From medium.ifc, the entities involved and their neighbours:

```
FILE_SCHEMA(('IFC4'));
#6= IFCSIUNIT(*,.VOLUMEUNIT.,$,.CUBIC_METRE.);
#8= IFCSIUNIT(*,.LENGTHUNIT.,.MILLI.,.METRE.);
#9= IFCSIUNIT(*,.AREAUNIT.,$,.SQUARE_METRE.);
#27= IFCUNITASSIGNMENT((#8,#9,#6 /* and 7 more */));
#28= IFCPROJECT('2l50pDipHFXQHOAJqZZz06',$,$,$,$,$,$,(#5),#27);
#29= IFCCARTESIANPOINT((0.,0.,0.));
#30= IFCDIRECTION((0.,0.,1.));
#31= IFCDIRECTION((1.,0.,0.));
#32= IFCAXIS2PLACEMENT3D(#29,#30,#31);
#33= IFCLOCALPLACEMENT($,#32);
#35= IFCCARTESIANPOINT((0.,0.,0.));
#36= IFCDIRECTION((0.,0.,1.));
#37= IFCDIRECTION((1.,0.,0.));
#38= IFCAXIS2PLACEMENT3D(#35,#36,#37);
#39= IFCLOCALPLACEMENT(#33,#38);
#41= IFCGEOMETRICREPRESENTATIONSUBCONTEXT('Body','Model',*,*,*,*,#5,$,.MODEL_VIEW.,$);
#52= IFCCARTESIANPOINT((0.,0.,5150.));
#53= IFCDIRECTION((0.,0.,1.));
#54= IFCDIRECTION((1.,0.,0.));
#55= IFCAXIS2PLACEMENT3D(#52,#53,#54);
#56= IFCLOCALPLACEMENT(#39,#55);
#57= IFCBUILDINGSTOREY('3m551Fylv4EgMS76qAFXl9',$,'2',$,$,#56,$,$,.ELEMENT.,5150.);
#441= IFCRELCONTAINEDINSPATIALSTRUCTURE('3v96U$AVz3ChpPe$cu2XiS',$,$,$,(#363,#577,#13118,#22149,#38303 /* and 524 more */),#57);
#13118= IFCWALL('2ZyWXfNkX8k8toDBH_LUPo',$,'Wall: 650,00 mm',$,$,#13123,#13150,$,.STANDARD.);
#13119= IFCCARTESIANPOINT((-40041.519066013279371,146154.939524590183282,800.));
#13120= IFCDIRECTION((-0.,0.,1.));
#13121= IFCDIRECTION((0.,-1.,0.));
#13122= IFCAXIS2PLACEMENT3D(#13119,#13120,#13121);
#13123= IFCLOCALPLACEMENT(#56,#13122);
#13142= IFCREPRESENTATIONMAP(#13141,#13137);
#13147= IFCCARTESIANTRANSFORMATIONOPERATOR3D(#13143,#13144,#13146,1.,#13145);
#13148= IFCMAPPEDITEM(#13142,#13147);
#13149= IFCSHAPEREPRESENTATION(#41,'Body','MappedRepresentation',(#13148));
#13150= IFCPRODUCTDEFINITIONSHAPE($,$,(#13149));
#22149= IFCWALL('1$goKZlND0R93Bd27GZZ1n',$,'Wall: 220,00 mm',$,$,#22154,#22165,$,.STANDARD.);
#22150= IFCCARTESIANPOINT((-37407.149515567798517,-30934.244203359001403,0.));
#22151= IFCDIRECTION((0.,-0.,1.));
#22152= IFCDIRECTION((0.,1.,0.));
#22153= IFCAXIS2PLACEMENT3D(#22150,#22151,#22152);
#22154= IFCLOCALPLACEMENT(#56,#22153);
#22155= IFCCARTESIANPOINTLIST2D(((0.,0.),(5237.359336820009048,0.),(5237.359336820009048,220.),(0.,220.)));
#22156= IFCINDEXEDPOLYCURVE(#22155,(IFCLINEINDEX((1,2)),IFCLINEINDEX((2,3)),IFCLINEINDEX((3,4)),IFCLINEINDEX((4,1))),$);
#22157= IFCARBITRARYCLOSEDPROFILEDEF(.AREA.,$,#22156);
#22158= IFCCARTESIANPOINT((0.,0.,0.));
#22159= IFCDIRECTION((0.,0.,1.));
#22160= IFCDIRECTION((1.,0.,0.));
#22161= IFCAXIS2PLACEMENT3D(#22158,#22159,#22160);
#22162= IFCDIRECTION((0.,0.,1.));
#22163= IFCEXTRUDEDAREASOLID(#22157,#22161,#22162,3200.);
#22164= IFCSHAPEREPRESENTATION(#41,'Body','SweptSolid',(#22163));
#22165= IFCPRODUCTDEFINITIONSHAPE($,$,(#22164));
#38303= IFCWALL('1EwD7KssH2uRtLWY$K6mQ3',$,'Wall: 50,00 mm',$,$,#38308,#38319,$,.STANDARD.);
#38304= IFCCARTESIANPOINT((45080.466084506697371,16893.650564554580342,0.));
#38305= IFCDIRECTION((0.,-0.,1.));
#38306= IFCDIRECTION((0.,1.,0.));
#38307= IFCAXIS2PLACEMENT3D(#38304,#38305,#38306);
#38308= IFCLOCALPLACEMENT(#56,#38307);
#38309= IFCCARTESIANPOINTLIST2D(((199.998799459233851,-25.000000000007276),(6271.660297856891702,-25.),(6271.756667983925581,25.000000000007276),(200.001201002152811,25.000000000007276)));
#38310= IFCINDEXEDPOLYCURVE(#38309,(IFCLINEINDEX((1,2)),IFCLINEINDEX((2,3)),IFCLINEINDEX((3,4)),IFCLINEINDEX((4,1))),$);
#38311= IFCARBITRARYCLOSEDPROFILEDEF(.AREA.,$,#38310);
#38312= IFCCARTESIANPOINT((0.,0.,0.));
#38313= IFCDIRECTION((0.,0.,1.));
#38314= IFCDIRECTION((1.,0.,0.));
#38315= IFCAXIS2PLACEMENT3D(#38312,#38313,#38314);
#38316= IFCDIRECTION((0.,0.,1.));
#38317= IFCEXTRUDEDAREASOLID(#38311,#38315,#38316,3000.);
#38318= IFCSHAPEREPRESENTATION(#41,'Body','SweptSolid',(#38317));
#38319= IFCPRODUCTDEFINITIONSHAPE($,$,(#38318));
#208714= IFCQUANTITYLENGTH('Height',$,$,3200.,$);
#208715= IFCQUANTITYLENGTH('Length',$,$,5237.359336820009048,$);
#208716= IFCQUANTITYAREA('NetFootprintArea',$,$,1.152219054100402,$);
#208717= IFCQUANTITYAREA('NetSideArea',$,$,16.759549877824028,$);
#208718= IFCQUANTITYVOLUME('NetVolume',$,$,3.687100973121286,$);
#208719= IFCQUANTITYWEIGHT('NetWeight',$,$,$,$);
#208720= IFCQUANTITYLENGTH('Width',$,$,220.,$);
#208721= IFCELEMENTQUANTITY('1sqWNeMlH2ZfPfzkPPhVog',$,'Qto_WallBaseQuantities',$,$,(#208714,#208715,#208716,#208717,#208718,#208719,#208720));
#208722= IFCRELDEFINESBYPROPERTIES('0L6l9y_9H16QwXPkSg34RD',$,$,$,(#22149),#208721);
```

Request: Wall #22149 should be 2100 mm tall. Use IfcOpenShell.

```python
import ifcopenshell
import ifcopenshell.api.pset
import ifcopenshell.geom
import ifcopenshell.util.element
import ifcopenshell.util.representation
import ifcopenshell.util.shape
import ifcopenshell.util.unit

model = ifcopenshell.open("medium.ifc")
area_scale = ifcopenshell.util.unit.calculate_unit_scale(model, "AREAUNIT")
volume_scale = ifcopenshell.util.unit.calculate_unit_scale(model, "VOLUMEUNIT")
settings = ifcopenshell.geom.settings()


def volume(element):
    """Net volume in cubic metres, openings subtracted."""
    shape = ifcopenshell.geom.create_shape(settings, element)
    return ifcopenshell.util.shape.get_volume(shape.geometry)


wall = model.by_guid("1$goKZlND0R93Bd27GZZ1n")
before = volume(wall)

body = ifcopenshell.util.representation.get_representation(wall, "Model", "Body")
solid = body.Items[0]
old_height = solid.Depth
solid.Depth = 2100.0
after = volume(wall)
thickness = 0.22  # wall thickness in metres

# Update the stored height, areas and volumes.
qto = model.by_id(ifcopenshell.util.element.get_pset(wall, "Qto_WallBaseQuantities", should_inherit=False)["id"])
ifcopenshell.api.pset.edit_qto(model, qto=qto, properties={
    "Height": solid.Depth,
    "NetSideArea": after / thickness / area_scale,
    "NetVolume": after / volume_scale,
})

print(f"height {old_height:g} -> {solid.Depth:g}, volume {before:.3f} -> {after:.3f} m3")

model.write("medium_updated.ifc")
```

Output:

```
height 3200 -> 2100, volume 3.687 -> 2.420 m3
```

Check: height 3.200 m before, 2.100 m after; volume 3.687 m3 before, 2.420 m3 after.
